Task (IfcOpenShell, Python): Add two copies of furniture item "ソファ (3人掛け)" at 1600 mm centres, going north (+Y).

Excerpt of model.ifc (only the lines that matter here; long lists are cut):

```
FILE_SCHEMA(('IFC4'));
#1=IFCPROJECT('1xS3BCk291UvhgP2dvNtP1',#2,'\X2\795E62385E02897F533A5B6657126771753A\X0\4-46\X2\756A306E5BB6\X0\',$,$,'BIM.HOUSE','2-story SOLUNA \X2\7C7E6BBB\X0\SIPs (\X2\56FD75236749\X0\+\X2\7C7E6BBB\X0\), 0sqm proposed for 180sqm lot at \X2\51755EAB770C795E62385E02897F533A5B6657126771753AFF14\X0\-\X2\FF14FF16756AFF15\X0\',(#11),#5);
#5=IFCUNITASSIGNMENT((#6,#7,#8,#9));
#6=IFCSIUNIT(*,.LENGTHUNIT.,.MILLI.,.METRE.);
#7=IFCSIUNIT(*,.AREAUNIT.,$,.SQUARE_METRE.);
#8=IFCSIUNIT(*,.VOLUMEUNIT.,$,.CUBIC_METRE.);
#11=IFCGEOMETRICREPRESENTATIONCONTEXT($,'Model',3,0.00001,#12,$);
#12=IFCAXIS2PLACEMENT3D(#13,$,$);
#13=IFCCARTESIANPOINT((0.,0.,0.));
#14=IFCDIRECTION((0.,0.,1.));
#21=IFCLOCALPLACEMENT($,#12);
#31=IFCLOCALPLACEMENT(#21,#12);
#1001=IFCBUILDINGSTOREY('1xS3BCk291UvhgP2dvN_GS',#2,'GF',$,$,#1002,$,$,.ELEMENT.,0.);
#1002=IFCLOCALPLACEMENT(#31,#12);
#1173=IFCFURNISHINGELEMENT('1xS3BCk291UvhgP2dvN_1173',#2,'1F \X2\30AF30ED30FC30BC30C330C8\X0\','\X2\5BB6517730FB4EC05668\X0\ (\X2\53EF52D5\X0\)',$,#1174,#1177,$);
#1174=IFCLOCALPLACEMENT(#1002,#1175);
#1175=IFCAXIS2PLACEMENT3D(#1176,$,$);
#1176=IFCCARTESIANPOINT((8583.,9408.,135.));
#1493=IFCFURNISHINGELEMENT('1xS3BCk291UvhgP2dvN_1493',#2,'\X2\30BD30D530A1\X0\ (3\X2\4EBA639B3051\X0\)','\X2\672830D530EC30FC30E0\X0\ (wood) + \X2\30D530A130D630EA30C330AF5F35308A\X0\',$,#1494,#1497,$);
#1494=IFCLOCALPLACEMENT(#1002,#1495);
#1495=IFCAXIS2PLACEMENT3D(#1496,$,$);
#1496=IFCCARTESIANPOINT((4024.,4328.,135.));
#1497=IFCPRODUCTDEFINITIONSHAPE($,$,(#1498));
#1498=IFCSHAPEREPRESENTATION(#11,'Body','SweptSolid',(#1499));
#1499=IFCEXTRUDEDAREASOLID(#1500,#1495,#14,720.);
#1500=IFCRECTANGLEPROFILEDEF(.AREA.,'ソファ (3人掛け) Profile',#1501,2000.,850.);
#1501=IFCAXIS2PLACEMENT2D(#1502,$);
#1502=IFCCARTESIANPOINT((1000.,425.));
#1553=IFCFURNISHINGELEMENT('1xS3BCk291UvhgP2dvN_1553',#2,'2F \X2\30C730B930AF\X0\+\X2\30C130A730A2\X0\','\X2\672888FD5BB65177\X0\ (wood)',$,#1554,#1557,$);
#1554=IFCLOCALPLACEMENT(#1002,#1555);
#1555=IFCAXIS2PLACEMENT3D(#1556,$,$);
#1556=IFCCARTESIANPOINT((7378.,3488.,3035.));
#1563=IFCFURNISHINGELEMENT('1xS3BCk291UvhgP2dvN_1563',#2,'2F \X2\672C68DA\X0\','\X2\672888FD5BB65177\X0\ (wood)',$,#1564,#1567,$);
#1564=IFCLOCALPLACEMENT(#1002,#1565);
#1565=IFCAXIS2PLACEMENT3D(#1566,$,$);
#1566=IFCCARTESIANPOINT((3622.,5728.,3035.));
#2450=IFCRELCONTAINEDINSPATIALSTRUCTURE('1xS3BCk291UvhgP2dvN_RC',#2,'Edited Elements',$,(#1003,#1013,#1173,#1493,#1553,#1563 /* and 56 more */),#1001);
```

```python
import numpy as np
import ifcopenshell
import ifcopenshell.api.geometry
import ifcopenshell.api.root
import ifcopenshell.util.element
import ifcopenshell.util.placement

model = ifcopenshell.open("model.ifc")


def reuse_history(source, copy):
    """copy_class also copies each property set's owner history, people and application; keep the originals."""
    for rel in copy.IsDefinedBy:
        if rel.is_a("IfcRelDefinesByProperties") and (history := rel.RelatingPropertyDefinition.OwnerHistory):
            rel.RelatingPropertyDefinition.OwnerHistory = source.OwnerHistory
            ifcopenshell.util.element.remove_deep2(model, history)


source = model.by_id(1493)
base = ifcopenshell.util.placement.get_local_placement(source.ObjectPlacement)
step = np.array([0.0, 1.0, 0.0]) * 1600.0

for i in range(1, 3):
    copy = ifcopenshell.api.root.copy_class(model, product=source)
    copy.Representation = ifcopenshell.util.element.copy_deep(
        model, source.Representation, exclude=["IfcGeometricRepresentationContext", "IfcRepresentationMap"]
    )
    reuse_history(source, copy)
    matrix = base.copy()
    matrix[:3, 3] += i * step
    print("added at", matrix[:3, 3].round(3) + 0.0)
    ifcopenshell.api.geometry.edit_object_placement(model, product=copy, matrix=matrix, is_si=False)

model.write("model_v2.ifc")
```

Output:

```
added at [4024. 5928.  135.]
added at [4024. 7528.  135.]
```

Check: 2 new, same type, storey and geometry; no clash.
